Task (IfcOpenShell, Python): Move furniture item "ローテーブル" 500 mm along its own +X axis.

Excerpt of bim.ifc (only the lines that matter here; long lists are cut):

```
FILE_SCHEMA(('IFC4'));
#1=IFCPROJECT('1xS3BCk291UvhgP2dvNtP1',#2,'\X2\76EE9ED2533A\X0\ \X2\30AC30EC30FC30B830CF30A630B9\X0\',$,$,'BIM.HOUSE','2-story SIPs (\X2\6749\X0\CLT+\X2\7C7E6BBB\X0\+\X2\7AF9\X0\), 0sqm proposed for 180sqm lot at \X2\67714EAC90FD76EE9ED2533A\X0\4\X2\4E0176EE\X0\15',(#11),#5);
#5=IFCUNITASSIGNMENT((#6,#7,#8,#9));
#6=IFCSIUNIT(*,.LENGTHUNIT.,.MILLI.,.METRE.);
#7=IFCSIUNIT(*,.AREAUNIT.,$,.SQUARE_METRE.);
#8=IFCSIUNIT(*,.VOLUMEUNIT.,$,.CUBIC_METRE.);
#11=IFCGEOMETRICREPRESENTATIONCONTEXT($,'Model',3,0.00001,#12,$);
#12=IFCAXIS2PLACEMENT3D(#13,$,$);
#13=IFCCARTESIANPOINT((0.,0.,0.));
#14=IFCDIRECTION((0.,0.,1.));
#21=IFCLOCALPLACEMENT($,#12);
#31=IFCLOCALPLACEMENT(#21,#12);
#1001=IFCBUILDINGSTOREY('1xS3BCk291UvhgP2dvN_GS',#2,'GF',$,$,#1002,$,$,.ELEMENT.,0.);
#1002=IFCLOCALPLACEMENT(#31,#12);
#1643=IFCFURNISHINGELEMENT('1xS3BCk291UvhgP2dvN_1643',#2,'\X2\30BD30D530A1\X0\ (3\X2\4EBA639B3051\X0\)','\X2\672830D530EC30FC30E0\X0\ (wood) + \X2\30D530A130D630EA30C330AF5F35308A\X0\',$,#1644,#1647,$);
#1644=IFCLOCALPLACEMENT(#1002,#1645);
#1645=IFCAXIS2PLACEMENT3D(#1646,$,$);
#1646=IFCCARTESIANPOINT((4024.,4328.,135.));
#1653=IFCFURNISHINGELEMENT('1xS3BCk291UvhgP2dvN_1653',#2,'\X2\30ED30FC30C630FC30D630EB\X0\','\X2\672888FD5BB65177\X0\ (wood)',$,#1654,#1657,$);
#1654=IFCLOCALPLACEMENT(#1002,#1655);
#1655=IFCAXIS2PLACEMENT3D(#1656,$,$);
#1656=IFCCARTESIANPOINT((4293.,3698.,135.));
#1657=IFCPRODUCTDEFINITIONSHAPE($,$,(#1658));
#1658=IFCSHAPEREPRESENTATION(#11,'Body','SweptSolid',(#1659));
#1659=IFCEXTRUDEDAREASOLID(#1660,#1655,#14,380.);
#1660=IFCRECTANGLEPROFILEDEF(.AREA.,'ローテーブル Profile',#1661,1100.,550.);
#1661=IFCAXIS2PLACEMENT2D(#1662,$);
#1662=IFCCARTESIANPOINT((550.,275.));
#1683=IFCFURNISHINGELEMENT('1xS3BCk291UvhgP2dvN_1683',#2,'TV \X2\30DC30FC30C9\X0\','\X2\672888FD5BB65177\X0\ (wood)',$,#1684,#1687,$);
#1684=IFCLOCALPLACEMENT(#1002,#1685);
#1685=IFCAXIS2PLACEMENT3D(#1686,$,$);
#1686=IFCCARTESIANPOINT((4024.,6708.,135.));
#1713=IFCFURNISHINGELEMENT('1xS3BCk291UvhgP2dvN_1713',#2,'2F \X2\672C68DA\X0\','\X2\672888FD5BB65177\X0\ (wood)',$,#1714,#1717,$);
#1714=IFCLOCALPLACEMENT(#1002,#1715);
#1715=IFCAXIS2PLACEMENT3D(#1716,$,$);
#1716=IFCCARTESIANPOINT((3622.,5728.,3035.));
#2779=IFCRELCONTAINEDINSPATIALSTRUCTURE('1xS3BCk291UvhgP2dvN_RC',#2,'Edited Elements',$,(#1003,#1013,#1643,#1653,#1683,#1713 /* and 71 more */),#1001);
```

```python
import ifcopenshell
import ifcopenshell.api.geometry
import ifcopenshell.util.placement
import ifcopenshell.util.unit

model = ifcopenshell.open("bim.ifc")
unit_scale = ifcopenshell.util.unit.calculate_unit_scale(model)

item = model.by_guid("1xS3BCk291UvhgP2dvN_1653")
matrix = ifcopenshell.util.placement.get_local_placement(item.ObjectPlacement)
matrix[:3, 3] += matrix[:3, 0] * 0.5 / unit_scale
ifcopenshell.api.geometry.edit_object_placement(model, product=item, matrix=matrix, is_si=False)

print(ifcopenshell.util.placement.get_local_placement(item.ObjectPlacement).round(3) + 0.0)

model.write("bim-out.ifc")
```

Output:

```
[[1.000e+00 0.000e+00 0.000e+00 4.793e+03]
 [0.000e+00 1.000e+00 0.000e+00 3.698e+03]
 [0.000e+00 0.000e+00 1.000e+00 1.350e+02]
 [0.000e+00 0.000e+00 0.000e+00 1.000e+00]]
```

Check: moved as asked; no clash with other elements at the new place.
